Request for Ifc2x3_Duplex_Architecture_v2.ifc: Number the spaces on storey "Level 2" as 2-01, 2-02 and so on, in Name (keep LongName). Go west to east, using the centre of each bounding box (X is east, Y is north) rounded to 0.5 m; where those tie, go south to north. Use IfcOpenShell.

First a look at what the model holds.

```python
import ifcopenshell
import ifcopenshell.util.element
import ifcopenshell.util.placement

model = ifcopenshell.open("Ifc2x3_Duplex_Architecture_v2.ifc")
print(model.schema)
storey = next(s for s in model.by_type("IfcBuildingStorey") if s.Name == "Level 2")
spaces = [e for e in ifcopenshell.util.element.get_decomposition(storey) if e.is_a("IfcSpace")]
for e in sorted(spaces, key=lambda e: e.id()):
    origin = ifcopenshell.util.placement.get_local_placement(e.ObjectPlacement)[:3, 3]
    print(e.id(), e.Name, e.LongName, origin.round(2) + 0.0, sep=" | ")
```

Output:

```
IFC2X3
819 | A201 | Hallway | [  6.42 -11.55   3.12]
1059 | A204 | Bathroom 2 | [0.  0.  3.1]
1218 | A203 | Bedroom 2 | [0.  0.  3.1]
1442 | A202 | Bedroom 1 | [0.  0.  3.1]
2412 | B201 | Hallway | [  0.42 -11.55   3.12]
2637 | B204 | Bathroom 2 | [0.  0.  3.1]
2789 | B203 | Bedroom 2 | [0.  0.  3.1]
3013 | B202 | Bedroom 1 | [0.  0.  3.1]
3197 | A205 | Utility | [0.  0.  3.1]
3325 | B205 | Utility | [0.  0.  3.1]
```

```python
import ifcopenshell
import ifcopenshell.geom
import ifcopenshell.util.element
import ifcopenshell.util.shape

model = ifcopenshell.open("Ifc2x3_Duplex_Architecture_v2.ifc")
settings = ifcopenshell.geom.settings()
settings.set("use-world-coords", True)


def centre(element):
    shape = ifcopenshell.geom.create_shape(settings, element)
    return ifcopenshell.util.shape.get_bbox_centroid(shape.geometry)


storey = next(s for s in model.by_type("IfcBuildingStorey") if s.Name == "Level 2")
spaces = [e for e in ifcopenshell.util.element.get_decomposition(storey) if e.is_a("IfcSpace")]

# Insertion points can sit at a corner or the storey origin, so sort by the geometry (in metres).
centres = {e: centre(e) for e in spaces}
spaces.sort(key=lambda e: (round(centres[e][0] / 0.5), centres[e][1]))

for i, e in enumerate(spaces, start=1):
    number = f"2-{i:02d}"
    e.Name = number
    print(e.id(), number)

model.write("Ifc2x3_Duplex_Architecture_v2_rev.ifc")
```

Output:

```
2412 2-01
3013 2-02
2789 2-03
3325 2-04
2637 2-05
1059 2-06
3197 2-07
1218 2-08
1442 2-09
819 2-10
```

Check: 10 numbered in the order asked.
